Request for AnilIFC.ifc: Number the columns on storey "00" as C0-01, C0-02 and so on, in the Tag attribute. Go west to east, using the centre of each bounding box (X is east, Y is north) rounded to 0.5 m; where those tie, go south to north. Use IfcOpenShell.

First a look at what the model holds.

```python
import ifcopenshell
import ifcopenshell.util.element
import ifcopenshell.util.placement

model = ifcopenshell.open("AnilIFC.ifc")
print(model.schema)
storey = next(s for s in model.by_type("IfcBuildingStorey") if s.Name == "00")
columns = [e for e in ifcopenshell.util.element.get_decomposition(storey) if e.is_a("IfcColumn")]
for e in sorted(columns, key=lambda e: e.id()):
    origin = ifcopenshell.util.placement.get_local_placement(e.ObjectPlacement)[:3, 3]
    print(e.id(), e.Tag, e.Name, origin.round(2) + 0.0, sep=" | ")
```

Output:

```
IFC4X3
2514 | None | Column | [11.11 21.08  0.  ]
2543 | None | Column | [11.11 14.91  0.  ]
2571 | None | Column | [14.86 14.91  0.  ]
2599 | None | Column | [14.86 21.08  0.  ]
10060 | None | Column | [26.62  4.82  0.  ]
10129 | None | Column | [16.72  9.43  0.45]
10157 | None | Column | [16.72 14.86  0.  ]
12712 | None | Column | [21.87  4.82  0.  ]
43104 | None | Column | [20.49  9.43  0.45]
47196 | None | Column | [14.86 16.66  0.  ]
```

```python
import ifcopenshell
import ifcopenshell.geom
import ifcopenshell.util.element
import ifcopenshell.util.shape

model = ifcopenshell.open("AnilIFC.ifc")
settings = ifcopenshell.geom.settings()
settings.set("use-world-coords", True)


def centre(element):
    shape = ifcopenshell.geom.create_shape(settings, element)
    return ifcopenshell.util.shape.get_bbox_centroid(shape.geometry)


storey = next(s for s in model.by_type("IfcBuildingStorey") if s.Name == "00")
columns = [e for e in ifcopenshell.util.element.get_decomposition(storey) if e.is_a("IfcColumn")]

# Insertion points can sit at a corner or the storey origin, so sort by the geometry (in metres).
centres = {e: centre(e) for e in columns}
columns.sort(key=lambda e: (round(centres[e][0] / 0.5), centres[e][1]))

for i, e in enumerate(columns, start=1):
    number = f"C0-{i:02d}"
    e.Tag = number
    print(e.id(), number)

model.write("AnilIFC_rev.ifc")
```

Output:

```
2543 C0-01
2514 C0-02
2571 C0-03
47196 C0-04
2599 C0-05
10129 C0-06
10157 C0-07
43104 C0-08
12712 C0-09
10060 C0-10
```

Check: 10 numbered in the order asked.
